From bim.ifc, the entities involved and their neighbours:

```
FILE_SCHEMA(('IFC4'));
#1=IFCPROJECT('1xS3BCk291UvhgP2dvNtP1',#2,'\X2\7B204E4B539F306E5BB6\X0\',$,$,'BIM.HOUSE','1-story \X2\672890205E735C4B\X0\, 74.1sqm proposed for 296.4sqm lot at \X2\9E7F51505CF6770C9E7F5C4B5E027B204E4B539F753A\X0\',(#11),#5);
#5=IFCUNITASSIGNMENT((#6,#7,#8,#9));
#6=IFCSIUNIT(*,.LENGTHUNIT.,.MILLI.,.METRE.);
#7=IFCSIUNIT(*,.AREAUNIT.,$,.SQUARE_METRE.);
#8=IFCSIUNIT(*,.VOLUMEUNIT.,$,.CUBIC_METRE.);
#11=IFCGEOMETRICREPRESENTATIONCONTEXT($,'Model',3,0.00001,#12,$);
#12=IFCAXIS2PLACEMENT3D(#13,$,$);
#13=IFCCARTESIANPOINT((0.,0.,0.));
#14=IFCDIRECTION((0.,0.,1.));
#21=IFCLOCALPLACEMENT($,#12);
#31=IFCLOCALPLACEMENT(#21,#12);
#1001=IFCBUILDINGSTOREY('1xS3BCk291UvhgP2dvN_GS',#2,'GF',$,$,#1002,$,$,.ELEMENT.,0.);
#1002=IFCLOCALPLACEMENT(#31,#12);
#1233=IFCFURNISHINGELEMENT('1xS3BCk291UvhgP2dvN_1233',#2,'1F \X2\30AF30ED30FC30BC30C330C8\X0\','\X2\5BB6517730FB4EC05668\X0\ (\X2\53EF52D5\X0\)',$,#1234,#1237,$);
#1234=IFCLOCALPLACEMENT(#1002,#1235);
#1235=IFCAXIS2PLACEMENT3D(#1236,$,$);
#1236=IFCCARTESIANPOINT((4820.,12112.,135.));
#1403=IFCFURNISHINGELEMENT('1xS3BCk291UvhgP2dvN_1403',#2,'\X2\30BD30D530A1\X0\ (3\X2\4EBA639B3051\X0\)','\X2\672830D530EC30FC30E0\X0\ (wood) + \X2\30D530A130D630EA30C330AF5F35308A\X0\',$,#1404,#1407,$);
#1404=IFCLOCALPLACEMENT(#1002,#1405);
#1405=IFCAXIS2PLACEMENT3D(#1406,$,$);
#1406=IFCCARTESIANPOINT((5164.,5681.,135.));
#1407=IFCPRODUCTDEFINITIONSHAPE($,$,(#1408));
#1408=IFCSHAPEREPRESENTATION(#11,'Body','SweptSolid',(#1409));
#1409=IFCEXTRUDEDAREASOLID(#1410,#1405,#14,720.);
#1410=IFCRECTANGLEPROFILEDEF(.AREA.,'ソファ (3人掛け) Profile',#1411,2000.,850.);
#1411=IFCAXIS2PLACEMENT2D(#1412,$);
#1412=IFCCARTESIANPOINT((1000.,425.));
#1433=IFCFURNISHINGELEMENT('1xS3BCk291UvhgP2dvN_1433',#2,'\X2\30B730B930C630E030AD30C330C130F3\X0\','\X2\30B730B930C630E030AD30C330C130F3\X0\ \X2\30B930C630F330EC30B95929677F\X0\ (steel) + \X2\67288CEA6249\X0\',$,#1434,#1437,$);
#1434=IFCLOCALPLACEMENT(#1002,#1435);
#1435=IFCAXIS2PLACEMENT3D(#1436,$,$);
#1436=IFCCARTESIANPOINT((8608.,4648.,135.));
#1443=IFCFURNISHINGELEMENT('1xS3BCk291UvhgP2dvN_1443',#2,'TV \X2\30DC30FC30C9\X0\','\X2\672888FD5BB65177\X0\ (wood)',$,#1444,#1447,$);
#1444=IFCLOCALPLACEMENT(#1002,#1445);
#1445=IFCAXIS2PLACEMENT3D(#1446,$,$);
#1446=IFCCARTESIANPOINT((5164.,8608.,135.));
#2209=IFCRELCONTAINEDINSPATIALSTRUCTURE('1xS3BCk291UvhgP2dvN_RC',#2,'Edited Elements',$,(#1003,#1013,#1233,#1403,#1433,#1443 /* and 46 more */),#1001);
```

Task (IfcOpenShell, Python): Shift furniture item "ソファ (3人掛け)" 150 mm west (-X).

```python
import ifcopenshell
import ifcopenshell.api.geometry
import ifcopenshell.util.placement

model = ifcopenshell.open("bim.ifc")

item = model.by_guid("1xS3BCk291UvhgP2dvN_1403")
matrix = ifcopenshell.util.placement.get_local_placement(item.ObjectPlacement)
matrix[0, 3] -= 150.0
ifcopenshell.api.geometry.edit_object_placement(model, product=item, matrix=matrix, is_si=False)

print(ifcopenshell.util.placement.get_local_placement(item.ObjectPlacement).round(3) + 0.0)

model.write("bim_updated.ifc")
```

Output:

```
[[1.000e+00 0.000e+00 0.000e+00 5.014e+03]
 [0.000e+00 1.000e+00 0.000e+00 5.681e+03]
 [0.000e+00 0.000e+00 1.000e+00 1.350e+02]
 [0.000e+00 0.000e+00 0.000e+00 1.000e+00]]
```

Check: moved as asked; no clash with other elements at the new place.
